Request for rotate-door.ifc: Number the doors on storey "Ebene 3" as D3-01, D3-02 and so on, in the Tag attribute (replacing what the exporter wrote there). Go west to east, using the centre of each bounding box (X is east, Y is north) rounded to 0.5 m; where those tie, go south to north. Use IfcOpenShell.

First a look at what the model holds.

```python
import ifcopenshell
import ifcopenshell.util.element
import ifcopenshell.util.placement

model = ifcopenshell.open("rotate-door.ifc")
print(model.schema)
storey = next(s for s in model.by_type("IfcBuildingStorey") if s.Name == "Ebene 3")
doors = [e for e in ifcopenshell.util.element.get_decomposition(storey) if e.is_a("IfcDoor")]
for e in sorted(doors, key=lambda e: e.id()):
    origin = ifcopenshell.util.placement.get_local_placement(e.ObjectPlacement)[:3, 3]
    print(e.id(), e.Tag, e.Name, origin.round(2) + 0.0, sep=" | ")
```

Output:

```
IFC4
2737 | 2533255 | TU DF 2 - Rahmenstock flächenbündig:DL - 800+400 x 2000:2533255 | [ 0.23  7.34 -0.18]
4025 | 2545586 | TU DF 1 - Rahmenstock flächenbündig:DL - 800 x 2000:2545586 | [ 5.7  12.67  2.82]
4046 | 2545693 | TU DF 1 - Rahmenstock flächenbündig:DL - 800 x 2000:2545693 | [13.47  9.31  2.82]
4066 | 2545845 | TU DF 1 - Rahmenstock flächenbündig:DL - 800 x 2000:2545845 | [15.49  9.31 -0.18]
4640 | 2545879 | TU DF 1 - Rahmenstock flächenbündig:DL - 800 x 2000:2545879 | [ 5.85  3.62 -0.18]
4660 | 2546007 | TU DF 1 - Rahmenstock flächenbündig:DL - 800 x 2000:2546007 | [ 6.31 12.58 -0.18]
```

```python
import ifcopenshell
import ifcopenshell.geom
import ifcopenshell.util.element
import ifcopenshell.util.shape

model = ifcopenshell.open("rotate-door.ifc")
settings = ifcopenshell.geom.settings()
settings.set("use-world-coords", True)


def centre(element):
    shape = ifcopenshell.geom.create_shape(settings, element)
    return ifcopenshell.util.shape.get_bbox_centroid(shape.geometry)


storey = next(s for s in model.by_type("IfcBuildingStorey") if s.Name == "Ebene 3")
doors = [e for e in ifcopenshell.util.element.get_decomposition(storey) if e.is_a("IfcDoor")]

# Insertion points can sit at a corner or the storey origin, so sort by the geometry (in metres).
centres = {e: centre(e) for e in doors}
doors.sort(key=lambda e: (round(centres[e][0] / 0.5), centres[e][1]))

for i, e in enumerate(doors, start=1):
    number = f"D3-{i:02d}"
    e.Tag = number
    print(e.id(), number)

model.write("rotate-door_edited.ifc")
```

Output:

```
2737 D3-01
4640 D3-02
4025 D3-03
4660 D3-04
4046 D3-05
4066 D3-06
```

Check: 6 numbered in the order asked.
